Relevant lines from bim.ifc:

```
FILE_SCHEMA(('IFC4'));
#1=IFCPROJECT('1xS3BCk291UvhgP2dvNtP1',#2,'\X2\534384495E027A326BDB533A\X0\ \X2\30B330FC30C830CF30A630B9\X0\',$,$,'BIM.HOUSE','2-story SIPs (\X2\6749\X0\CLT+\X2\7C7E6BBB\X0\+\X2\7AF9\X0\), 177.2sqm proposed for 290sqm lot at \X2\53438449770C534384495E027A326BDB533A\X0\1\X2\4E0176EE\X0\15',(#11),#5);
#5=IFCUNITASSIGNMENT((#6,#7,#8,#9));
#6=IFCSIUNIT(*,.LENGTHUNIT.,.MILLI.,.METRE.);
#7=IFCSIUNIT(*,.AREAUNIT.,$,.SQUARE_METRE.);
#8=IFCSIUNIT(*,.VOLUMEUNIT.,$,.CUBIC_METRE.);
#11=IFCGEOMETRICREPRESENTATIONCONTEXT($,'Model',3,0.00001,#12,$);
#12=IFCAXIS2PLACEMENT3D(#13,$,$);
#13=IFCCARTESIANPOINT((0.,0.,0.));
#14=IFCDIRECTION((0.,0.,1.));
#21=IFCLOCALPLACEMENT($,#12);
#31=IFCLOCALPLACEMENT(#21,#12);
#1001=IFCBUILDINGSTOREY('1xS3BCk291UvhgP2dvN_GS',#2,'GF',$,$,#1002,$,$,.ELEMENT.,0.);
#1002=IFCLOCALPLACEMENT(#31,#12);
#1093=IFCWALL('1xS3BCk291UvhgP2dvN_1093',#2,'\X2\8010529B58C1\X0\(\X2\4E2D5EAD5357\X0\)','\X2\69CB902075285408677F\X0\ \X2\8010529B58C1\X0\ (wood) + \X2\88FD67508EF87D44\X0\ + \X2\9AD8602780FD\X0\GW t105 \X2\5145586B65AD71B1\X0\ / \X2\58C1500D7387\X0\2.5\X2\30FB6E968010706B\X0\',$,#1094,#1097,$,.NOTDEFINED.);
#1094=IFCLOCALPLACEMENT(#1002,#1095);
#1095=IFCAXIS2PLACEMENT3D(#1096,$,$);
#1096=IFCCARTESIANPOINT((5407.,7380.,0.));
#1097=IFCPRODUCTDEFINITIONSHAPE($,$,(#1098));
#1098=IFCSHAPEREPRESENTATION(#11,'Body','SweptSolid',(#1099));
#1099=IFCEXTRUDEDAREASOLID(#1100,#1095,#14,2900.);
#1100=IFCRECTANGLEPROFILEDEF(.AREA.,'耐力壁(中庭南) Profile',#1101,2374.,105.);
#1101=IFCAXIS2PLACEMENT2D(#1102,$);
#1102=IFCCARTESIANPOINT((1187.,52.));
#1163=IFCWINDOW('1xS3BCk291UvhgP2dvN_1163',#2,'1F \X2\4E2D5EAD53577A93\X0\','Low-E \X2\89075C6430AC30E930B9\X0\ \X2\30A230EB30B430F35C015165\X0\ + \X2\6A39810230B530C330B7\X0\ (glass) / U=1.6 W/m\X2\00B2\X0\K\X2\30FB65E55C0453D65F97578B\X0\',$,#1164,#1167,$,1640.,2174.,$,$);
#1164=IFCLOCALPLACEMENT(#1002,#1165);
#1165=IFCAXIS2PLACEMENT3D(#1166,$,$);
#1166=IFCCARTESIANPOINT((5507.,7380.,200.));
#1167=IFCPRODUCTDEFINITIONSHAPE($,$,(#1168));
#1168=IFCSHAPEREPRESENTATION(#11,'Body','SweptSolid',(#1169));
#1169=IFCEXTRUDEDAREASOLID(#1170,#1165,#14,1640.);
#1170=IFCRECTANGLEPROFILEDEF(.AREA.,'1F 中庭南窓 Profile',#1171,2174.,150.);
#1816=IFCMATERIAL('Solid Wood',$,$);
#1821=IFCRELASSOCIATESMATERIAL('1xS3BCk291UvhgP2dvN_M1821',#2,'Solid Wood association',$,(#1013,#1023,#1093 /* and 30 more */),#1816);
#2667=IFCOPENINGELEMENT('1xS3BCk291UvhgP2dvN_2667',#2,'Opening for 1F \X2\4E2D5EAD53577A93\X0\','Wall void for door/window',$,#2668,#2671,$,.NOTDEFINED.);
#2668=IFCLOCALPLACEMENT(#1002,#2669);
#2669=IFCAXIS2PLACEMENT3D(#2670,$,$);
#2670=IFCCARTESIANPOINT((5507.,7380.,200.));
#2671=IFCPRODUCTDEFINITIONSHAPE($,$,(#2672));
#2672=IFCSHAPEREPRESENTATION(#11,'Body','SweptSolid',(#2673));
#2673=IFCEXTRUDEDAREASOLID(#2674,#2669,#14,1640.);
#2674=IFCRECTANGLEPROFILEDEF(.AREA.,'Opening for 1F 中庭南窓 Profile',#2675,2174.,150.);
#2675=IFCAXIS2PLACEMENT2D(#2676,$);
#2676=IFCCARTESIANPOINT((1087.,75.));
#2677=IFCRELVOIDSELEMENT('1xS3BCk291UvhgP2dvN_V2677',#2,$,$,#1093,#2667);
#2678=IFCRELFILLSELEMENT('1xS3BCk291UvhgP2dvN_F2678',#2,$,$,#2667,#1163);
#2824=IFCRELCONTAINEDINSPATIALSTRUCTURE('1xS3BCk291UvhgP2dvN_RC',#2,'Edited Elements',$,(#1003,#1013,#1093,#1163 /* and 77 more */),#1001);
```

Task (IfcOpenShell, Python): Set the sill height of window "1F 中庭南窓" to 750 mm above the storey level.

```python
import numpy as np
import ifcopenshell
import ifcopenshell.api.geometry
import ifcopenshell.geom
import ifcopenshell.util.element
import ifcopenshell.util.placement
import ifcopenshell.util.shape
import ifcopenshell.util.unit

model = ifcopenshell.open("bim.ifc")
unit_scale = ifcopenshell.util.unit.calculate_unit_scale(model)

window = model.by_guid("1xS3BCk291UvhgP2dvN_1163")
opening = window.FillsVoids[0].RelatingOpeningElement
storey = ifcopenshell.util.element.get_container(window, ifc_class="IfcBuildingStorey")
level = ifcopenshell.util.placement.get_local_placement(storey.ObjectPlacement)[2, 3]

# The opening's origin need not be at the sill, so measure its lowest point.
shape = ifcopenshell.geom.create_shape(ifcopenshell.geom.settings(), opening)
bottom = ifcopenshell.util.shape.get_shape_bottom_elevation(shape, shape.geometry) / unit_scale
dz = level + 750.0 - bottom

shift = np.array([0.0, 0.0, dz])
# The window is not placed relative to its opening, so move both.
for product in (opening, window):
    matrix = ifcopenshell.util.placement.get_local_placement(product.ObjectPlacement)
    matrix[:3, 3] += shift
    ifcopenshell.api.geometry.edit_object_placement(model, product=product, matrix=matrix, is_si=False)

print(f"moved by {dz * unit_scale:+.3f} m")

model.write("bim_rev.ifc")
```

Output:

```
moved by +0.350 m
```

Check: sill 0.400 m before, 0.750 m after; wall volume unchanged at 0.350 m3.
